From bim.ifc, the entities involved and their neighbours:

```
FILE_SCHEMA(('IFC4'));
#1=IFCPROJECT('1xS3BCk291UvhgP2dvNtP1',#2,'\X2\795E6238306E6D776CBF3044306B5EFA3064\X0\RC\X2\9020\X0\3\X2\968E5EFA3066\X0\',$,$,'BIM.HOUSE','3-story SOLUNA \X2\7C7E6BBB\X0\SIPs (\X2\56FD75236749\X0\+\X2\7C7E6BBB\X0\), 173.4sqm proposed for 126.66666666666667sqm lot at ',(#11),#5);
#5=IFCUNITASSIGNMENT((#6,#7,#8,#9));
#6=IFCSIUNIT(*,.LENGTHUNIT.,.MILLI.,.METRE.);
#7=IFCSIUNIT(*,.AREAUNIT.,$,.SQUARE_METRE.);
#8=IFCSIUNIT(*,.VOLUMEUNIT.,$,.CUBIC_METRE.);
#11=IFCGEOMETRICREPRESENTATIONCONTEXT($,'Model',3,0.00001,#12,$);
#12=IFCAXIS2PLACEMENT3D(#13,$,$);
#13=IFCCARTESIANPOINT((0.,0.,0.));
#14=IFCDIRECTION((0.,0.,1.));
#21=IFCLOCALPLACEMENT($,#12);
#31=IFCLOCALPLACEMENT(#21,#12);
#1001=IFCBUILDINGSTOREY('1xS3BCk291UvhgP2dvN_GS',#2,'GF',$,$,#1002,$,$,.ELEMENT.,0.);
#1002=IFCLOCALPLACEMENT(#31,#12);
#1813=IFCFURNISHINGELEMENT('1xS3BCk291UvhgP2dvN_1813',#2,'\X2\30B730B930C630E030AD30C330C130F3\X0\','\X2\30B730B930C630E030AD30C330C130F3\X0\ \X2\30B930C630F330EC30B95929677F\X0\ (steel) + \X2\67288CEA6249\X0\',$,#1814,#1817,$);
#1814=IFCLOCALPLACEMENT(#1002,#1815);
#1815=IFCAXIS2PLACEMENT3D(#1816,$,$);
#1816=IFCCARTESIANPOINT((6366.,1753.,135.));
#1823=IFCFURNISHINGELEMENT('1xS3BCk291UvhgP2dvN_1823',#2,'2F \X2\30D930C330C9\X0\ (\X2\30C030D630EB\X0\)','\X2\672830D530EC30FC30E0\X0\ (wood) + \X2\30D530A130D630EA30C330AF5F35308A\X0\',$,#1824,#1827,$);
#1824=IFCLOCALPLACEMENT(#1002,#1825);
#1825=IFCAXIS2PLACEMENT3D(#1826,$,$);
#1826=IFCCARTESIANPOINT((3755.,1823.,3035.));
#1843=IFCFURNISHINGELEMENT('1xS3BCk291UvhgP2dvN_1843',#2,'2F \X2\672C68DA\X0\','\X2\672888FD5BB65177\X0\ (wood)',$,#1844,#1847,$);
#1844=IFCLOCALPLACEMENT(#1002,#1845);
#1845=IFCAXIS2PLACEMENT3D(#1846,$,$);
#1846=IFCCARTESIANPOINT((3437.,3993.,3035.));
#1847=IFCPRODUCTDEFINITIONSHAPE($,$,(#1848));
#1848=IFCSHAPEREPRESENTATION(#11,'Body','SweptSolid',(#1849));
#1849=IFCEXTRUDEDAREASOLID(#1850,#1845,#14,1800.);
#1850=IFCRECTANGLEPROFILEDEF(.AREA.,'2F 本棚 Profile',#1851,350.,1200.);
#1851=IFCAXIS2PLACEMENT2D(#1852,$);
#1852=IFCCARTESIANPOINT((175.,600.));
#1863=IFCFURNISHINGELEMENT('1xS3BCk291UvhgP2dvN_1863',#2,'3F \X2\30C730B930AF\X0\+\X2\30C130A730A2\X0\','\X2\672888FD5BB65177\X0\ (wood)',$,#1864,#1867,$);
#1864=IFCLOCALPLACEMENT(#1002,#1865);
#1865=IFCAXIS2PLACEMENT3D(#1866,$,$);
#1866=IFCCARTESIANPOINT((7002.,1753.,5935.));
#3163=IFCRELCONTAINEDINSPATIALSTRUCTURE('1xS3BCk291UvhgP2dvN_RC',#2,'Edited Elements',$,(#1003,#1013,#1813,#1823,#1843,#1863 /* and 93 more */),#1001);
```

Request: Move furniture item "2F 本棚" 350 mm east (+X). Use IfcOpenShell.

```python
import ifcopenshell
import ifcopenshell.api.geometry
import ifcopenshell.util.placement
import ifcopenshell.util.unit

model = ifcopenshell.open("bim.ifc")
unit_scale = ifcopenshell.util.unit.calculate_unit_scale(model)

item = model.by_guid("1xS3BCk291UvhgP2dvN_1843")
matrix = ifcopenshell.util.placement.get_local_placement(item.ObjectPlacement)
matrix[0, 3] += 0.35 / unit_scale
ifcopenshell.api.geometry.edit_object_placement(model, product=item, matrix=matrix, is_si=False)

print(ifcopenshell.util.placement.get_local_placement(item.ObjectPlacement).round(3) + 0.0)

model.write("bim_updated.ifc")
```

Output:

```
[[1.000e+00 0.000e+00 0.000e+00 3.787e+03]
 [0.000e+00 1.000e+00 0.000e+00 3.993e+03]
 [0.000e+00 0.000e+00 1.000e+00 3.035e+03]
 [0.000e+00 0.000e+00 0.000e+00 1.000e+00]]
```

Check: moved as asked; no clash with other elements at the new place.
